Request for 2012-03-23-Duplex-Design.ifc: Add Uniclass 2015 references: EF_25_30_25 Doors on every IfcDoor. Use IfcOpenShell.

First a look at what the model holds.

```python
import ifcopenshell

model = ifcopenshell.open("2012-03-23-Duplex-Design.ifc")
print(model.schema)
print("classifications:", [c.Name for c in model.by_type("IfcClassification")])
for ifc_class in ("IfcDoor", "IfcRoof", "IfcStair", "IfcWall", "IfcWindow"):
    print(ifc_class, len(model.by_type(ifc_class)))
```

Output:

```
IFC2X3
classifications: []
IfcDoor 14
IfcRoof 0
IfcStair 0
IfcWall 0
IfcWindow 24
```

```python
import ifcopenshell
import ifcopenshell.api.classification

model = ifcopenshell.open("2012-03-23-Duplex-Design.ifc")

# IFC2X3 requires Source and Edition and has no link from the project to the system.
system = model.create_entity("IfcClassification", Source="NBS", Edition="2015", Name="Uniclass 2015")

codes = {
    "IfcDoor": ("EF_25_30_25", "Doors"),
}
for ifc_class, (code, name) in codes.items():
    products = model.by_type(ifc_class)
    ifcopenshell.api.classification.add_reference(
        model, products=products, classification=system, identification=code, name=name
    )
    print(code, len(products))

model.write("2012-03-23-Duplex-Design_edited.ifc")
```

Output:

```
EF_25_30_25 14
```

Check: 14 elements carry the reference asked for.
